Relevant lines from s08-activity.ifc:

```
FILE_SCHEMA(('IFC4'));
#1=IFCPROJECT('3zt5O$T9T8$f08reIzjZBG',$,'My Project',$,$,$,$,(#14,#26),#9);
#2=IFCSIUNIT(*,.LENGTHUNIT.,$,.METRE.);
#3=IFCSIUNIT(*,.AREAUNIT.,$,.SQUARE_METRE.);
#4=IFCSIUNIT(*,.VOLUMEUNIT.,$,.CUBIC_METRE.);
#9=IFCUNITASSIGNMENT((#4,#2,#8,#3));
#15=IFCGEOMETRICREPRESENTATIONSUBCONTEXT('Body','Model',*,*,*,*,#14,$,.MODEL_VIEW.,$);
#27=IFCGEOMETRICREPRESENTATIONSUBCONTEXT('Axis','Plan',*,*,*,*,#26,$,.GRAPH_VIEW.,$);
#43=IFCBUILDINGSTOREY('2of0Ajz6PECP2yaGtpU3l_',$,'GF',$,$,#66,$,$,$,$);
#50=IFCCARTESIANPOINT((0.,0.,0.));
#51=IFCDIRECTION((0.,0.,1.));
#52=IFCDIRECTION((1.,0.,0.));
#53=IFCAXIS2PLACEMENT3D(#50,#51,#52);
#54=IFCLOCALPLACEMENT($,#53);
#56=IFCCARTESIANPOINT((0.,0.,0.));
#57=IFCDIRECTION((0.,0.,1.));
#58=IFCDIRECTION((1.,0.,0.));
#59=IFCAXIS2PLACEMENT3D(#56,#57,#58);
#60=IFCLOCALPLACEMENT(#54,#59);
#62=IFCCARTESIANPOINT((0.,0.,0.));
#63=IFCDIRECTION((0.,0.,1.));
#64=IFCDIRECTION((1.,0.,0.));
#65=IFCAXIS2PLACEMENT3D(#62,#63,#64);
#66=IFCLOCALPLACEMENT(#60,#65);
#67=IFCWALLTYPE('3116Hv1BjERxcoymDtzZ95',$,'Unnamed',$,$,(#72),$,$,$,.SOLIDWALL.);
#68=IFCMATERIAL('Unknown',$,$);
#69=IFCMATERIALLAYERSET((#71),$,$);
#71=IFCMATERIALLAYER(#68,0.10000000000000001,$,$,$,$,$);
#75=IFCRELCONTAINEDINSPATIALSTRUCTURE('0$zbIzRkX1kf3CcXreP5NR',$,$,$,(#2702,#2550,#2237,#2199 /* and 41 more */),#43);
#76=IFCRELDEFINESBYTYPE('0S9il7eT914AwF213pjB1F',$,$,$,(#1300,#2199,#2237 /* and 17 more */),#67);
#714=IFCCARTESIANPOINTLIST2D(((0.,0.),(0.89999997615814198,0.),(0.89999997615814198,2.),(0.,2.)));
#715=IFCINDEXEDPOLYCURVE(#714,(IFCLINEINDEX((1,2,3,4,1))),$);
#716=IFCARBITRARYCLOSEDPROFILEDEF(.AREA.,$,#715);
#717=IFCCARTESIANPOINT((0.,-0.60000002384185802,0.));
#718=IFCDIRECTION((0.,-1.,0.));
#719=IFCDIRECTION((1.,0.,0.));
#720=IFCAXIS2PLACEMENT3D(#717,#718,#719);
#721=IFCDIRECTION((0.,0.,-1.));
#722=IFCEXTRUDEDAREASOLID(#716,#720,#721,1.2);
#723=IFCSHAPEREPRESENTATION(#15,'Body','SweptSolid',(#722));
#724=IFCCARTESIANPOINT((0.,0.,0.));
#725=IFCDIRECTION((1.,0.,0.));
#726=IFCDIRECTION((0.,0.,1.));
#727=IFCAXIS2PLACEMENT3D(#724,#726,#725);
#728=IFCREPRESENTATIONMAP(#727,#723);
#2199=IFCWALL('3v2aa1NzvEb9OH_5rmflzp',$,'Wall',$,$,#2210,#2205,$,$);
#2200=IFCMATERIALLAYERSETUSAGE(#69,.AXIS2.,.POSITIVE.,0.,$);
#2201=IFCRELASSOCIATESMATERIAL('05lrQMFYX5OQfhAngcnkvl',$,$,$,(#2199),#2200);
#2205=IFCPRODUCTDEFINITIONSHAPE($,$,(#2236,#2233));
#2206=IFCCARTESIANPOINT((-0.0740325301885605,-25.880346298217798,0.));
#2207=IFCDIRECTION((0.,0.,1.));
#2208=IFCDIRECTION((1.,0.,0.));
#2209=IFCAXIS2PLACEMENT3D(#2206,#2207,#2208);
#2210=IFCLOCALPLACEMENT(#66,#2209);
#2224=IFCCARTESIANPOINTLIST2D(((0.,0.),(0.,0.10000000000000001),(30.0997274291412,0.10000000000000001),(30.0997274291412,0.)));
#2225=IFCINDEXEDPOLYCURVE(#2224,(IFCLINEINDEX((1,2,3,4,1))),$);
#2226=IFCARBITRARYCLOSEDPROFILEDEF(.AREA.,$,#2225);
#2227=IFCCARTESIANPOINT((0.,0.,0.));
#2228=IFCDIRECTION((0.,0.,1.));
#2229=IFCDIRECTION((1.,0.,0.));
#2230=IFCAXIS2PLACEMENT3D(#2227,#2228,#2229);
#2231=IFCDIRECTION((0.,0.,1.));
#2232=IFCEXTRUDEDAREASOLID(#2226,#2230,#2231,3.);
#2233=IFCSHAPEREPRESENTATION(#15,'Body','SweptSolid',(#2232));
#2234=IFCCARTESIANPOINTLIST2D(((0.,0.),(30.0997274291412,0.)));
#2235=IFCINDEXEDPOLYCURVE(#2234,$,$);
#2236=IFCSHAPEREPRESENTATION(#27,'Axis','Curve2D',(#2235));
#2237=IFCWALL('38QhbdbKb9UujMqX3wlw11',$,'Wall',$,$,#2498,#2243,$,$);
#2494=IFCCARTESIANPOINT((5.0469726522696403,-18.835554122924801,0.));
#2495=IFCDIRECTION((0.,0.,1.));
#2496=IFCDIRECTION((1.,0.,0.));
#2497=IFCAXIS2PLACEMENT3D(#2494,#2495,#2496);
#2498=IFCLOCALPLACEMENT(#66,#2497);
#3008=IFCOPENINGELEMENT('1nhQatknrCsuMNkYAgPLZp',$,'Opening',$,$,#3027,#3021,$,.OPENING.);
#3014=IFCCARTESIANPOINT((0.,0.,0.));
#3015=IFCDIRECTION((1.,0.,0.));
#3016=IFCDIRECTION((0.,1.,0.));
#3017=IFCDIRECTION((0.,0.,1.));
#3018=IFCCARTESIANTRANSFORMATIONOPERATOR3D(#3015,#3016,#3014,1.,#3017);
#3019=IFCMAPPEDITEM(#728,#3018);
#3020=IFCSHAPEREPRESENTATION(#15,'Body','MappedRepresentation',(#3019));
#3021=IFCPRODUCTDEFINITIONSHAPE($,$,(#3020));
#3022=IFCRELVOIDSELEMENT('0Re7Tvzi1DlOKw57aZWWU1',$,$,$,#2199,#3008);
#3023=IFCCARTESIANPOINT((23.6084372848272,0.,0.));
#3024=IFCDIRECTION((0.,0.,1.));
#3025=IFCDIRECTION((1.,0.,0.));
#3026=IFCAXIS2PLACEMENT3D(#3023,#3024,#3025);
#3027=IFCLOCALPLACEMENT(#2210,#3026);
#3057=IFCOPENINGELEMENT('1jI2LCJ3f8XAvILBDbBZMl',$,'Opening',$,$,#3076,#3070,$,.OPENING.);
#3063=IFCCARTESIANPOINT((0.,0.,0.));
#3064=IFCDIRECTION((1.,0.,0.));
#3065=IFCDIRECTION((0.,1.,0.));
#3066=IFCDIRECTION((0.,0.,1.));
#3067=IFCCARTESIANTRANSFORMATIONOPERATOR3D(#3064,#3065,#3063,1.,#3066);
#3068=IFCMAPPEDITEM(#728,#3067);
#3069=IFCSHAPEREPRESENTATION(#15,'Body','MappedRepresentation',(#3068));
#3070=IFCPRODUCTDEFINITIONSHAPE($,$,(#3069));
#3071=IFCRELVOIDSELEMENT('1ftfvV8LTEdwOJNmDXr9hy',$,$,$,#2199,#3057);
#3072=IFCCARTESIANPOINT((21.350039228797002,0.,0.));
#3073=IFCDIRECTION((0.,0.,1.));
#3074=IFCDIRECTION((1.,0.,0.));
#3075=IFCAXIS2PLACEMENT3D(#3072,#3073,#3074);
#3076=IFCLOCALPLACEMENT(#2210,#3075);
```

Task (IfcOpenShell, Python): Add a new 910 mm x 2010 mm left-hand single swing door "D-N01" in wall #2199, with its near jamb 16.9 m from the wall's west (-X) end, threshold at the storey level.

```python
import numpy as np
import ifcopenshell
import ifcopenshell.api.feature
import ifcopenshell.api.geometry
import ifcopenshell.api.root
import ifcopenshell.api.spatial
import ifcopenshell.geom
import ifcopenshell.util.element
import ifcopenshell.util.placement
import ifcopenshell.util.representation
import ifcopenshell.util.shape
import ifcopenshell.util.unit

model = ifcopenshell.open("s08-activity.ifc")
unit_scale = ifcopenshell.util.unit.calculate_unit_scale(model)
settings = ifcopenshell.geom.settings()


def volume(element):
    """Net volume in cubic metres, openings subtracted."""
    shape = ifcopenshell.geom.create_shape(settings, element)
    return ifcopenshell.util.shape.get_volume(shape.geometry)


wall = model.by_guid("3v2aa1NzvEb9OH_5rmflzp")
storey = ifcopenshell.util.element.get_container(wall, ifc_class="IfcBuildingStorey")
context = ifcopenshell.util.representation.get_context(model, "Model", "Body", "MODEL_VIEW")
before = volume(wall)

width, height, from_end, sill = 0.91, 2.01, 16.9, 0.0  # metres

# The wall runs along its own X axis, and the end named is its -X end.
wall_shape = ifcopenshell.geom.create_shape(settings, wall)
x, y, z = ifcopenshell.util.shape.get_vertices(wall_shape.geometry).T
start = x.min() + from_end
face, thickness = float(y.min()), float(y.max() - y.min())
wall_matrix = ifcopenshell.util.placement.get_local_placement(wall.ObjectPlacement)
level = ifcopenshell.util.placement.get_local_placement(storey.ObjectPlacement)[2, 3]


def in_wall(x, y):
    """Placement at x, y metres in the wall's axes, at sill height."""
    matrix = wall_matrix.copy()
    matrix[:, 3] = wall_matrix @ np.array([x / unit_scale, y / unit_scale, 0.0, 1.0])
    matrix[2, 3] = level + sill / unit_scale
    return matrix


# Opening: a box that overshoots both wall faces by 50 mm.
opening = ifcopenshell.api.root.create_entity(model, ifc_class="IfcOpeningElement", predefined_type="OPENING")
box = ifcopenshell.api.geometry.add_wall_representation(
    model, context=context, length=width, height=height, thickness=thickness + 0.1
)
ifcopenshell.api.geometry.assign_representation(model, product=opening, representation=box)
ifcopenshell.api.geometry.edit_object_placement(model, product=opening, matrix=in_wall(start, face - 0.05), is_si=False)
ifcopenshell.api.feature.add_feature(model, feature=opening, element=wall)

door = ifcopenshell.api.root.create_entity(model, ifc_class="IfcDoor", name="D-N01", predefined_type="DOOR")
door.OverallWidth, door.OverallHeight = width / unit_scale, height / unit_scale
door.OperationType = "SINGLE_SWING_LEFT"
body = ifcopenshell.api.geometry.add_door_representation(
    model,
    context=context,
    overall_width=door.OverallWidth,
    overall_height=door.OverallHeight,
    operation_type="SINGLE_SWING_LEFT",
    lining_properties={"LiningDepth": thickness / unit_scale, "ThresholdDepth": thickness / unit_scale},
)
ifcopenshell.api.geometry.assign_representation(model, product=door, representation=body)
ifcopenshell.api.spatial.assign_container(model, products=[door], relating_structure=storey)
ifcopenshell.api.feature.add_filling(model, opening=opening, element=door)

# The lining spans the wall, so the door starts at the wall face.
ifcopenshell.api.geometry.edit_object_placement(model, product=door, matrix=in_wall(start, face), is_si=False)

after = volume(wall)

print(f"wall volume {before:.3f} -> {after:.3f} m3")

model.write("s08-activity_v2.ifc")
```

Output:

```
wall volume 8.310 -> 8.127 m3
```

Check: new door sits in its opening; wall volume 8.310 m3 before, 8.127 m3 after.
